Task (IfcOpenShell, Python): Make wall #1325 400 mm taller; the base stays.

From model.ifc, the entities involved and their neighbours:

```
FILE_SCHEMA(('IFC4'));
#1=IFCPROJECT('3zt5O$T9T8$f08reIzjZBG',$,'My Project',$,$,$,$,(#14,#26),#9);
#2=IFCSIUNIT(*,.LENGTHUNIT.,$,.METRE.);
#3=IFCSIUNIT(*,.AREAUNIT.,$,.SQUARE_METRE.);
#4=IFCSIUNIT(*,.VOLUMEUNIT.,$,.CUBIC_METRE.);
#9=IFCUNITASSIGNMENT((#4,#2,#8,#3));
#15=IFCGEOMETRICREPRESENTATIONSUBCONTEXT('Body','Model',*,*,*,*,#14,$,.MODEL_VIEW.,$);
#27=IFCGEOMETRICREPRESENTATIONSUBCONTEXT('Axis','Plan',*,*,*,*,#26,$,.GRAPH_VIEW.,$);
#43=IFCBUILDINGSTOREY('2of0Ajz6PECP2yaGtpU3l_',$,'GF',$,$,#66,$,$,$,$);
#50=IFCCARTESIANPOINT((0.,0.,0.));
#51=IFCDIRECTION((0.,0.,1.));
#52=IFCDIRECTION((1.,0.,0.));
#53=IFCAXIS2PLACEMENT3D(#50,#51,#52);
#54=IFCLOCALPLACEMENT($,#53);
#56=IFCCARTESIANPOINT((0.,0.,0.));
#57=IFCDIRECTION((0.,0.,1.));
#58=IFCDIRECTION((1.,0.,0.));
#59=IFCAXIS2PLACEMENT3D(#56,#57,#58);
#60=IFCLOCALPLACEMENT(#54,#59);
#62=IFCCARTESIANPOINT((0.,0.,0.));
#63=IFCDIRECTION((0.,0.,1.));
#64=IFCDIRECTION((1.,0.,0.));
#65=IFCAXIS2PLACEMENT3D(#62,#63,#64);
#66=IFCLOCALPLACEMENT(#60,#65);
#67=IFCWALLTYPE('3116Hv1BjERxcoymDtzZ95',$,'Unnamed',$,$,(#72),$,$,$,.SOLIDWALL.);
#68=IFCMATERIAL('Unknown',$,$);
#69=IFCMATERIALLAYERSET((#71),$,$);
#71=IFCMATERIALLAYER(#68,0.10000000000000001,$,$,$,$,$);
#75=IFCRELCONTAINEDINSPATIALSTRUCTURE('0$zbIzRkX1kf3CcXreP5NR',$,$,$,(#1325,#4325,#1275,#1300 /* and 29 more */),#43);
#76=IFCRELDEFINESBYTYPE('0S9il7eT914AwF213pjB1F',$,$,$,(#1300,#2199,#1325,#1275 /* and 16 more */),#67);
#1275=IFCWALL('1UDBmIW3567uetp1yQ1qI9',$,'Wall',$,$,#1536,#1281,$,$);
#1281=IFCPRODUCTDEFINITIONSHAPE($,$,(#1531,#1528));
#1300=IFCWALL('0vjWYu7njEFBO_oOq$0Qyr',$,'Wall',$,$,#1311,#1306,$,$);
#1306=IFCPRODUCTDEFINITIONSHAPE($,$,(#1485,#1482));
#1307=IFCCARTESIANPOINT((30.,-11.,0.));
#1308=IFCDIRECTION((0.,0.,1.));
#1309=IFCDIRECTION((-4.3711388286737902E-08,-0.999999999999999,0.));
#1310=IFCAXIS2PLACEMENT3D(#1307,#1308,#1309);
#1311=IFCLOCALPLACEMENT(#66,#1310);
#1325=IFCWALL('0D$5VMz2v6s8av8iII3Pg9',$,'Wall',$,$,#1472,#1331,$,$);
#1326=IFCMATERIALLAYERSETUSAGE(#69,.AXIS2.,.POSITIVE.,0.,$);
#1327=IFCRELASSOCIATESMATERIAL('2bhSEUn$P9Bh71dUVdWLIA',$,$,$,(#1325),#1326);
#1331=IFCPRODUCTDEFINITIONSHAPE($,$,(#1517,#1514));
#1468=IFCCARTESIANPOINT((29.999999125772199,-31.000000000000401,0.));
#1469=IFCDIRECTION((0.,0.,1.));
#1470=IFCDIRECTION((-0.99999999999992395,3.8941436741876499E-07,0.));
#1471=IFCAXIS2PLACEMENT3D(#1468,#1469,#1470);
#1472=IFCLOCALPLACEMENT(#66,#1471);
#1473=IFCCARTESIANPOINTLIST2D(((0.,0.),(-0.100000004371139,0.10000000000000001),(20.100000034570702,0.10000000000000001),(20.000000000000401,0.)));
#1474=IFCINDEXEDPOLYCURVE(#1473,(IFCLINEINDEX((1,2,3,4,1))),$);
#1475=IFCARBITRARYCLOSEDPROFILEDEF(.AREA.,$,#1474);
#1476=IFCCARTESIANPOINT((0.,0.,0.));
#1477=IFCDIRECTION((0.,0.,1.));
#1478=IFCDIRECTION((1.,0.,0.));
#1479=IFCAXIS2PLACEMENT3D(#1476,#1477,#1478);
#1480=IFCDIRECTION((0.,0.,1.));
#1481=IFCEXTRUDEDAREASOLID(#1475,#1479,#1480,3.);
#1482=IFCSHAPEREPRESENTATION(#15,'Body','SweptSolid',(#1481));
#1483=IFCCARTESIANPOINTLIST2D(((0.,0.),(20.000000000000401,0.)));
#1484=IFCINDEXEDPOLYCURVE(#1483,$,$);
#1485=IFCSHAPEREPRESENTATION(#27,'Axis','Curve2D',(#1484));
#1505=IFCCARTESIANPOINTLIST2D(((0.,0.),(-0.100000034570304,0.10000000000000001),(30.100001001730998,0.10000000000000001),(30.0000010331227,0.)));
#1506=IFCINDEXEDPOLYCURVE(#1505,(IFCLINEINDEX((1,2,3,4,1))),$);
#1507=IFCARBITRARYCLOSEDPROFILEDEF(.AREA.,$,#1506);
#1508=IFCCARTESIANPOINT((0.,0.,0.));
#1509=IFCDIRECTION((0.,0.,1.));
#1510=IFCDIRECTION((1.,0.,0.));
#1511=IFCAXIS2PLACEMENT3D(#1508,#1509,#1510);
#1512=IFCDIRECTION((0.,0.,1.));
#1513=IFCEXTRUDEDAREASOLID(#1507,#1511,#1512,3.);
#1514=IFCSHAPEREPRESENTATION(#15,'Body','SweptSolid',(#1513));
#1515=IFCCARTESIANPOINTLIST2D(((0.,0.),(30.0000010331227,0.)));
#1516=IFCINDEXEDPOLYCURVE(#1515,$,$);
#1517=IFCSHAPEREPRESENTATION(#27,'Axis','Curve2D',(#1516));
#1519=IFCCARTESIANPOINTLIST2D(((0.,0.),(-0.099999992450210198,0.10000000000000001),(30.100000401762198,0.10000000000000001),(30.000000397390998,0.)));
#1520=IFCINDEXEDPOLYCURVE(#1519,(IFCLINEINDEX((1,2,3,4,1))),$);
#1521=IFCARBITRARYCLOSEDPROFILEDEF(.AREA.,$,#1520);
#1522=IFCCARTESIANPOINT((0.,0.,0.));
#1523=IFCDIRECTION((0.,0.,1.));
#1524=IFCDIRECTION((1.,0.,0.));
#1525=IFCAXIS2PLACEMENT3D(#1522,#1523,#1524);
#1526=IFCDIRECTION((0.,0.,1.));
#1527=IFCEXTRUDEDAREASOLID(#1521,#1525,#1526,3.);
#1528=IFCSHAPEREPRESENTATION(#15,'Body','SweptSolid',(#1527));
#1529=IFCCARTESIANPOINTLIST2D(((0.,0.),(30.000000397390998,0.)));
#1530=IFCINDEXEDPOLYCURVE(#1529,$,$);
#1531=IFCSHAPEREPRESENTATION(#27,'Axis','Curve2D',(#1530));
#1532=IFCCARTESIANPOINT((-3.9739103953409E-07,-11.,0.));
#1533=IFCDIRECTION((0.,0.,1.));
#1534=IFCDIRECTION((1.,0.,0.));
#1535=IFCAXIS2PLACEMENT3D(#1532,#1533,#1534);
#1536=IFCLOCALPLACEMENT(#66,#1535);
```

```python
import ifcopenshell
import ifcopenshell.geom
import ifcopenshell.util.representation
import ifcopenshell.util.shape

model = ifcopenshell.open("model.ifc")
settings = ifcopenshell.geom.settings()


def volume(element):
    """Net volume in cubic metres, openings subtracted."""
    shape = ifcopenshell.geom.create_shape(settings, element)
    return ifcopenshell.util.shape.get_volume(shape.geometry)


wall = model.by_guid("0D$5VMz2v6s8av8iII3Pg9")
before = volume(wall)

body = ifcopenshell.util.representation.get_representation(wall, "Model", "Body")
solid = body.Items[0]
old_height = solid.Depth
solid.Depth += 0.4
after = volume(wall)

print(f"height {old_height:g} -> {solid.Depth:g}, volume {before:.3f} -> {after:.3f} m3")

model.write("model_edited.ifc")
```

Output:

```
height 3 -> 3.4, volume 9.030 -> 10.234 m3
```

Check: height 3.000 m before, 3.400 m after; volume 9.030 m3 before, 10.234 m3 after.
